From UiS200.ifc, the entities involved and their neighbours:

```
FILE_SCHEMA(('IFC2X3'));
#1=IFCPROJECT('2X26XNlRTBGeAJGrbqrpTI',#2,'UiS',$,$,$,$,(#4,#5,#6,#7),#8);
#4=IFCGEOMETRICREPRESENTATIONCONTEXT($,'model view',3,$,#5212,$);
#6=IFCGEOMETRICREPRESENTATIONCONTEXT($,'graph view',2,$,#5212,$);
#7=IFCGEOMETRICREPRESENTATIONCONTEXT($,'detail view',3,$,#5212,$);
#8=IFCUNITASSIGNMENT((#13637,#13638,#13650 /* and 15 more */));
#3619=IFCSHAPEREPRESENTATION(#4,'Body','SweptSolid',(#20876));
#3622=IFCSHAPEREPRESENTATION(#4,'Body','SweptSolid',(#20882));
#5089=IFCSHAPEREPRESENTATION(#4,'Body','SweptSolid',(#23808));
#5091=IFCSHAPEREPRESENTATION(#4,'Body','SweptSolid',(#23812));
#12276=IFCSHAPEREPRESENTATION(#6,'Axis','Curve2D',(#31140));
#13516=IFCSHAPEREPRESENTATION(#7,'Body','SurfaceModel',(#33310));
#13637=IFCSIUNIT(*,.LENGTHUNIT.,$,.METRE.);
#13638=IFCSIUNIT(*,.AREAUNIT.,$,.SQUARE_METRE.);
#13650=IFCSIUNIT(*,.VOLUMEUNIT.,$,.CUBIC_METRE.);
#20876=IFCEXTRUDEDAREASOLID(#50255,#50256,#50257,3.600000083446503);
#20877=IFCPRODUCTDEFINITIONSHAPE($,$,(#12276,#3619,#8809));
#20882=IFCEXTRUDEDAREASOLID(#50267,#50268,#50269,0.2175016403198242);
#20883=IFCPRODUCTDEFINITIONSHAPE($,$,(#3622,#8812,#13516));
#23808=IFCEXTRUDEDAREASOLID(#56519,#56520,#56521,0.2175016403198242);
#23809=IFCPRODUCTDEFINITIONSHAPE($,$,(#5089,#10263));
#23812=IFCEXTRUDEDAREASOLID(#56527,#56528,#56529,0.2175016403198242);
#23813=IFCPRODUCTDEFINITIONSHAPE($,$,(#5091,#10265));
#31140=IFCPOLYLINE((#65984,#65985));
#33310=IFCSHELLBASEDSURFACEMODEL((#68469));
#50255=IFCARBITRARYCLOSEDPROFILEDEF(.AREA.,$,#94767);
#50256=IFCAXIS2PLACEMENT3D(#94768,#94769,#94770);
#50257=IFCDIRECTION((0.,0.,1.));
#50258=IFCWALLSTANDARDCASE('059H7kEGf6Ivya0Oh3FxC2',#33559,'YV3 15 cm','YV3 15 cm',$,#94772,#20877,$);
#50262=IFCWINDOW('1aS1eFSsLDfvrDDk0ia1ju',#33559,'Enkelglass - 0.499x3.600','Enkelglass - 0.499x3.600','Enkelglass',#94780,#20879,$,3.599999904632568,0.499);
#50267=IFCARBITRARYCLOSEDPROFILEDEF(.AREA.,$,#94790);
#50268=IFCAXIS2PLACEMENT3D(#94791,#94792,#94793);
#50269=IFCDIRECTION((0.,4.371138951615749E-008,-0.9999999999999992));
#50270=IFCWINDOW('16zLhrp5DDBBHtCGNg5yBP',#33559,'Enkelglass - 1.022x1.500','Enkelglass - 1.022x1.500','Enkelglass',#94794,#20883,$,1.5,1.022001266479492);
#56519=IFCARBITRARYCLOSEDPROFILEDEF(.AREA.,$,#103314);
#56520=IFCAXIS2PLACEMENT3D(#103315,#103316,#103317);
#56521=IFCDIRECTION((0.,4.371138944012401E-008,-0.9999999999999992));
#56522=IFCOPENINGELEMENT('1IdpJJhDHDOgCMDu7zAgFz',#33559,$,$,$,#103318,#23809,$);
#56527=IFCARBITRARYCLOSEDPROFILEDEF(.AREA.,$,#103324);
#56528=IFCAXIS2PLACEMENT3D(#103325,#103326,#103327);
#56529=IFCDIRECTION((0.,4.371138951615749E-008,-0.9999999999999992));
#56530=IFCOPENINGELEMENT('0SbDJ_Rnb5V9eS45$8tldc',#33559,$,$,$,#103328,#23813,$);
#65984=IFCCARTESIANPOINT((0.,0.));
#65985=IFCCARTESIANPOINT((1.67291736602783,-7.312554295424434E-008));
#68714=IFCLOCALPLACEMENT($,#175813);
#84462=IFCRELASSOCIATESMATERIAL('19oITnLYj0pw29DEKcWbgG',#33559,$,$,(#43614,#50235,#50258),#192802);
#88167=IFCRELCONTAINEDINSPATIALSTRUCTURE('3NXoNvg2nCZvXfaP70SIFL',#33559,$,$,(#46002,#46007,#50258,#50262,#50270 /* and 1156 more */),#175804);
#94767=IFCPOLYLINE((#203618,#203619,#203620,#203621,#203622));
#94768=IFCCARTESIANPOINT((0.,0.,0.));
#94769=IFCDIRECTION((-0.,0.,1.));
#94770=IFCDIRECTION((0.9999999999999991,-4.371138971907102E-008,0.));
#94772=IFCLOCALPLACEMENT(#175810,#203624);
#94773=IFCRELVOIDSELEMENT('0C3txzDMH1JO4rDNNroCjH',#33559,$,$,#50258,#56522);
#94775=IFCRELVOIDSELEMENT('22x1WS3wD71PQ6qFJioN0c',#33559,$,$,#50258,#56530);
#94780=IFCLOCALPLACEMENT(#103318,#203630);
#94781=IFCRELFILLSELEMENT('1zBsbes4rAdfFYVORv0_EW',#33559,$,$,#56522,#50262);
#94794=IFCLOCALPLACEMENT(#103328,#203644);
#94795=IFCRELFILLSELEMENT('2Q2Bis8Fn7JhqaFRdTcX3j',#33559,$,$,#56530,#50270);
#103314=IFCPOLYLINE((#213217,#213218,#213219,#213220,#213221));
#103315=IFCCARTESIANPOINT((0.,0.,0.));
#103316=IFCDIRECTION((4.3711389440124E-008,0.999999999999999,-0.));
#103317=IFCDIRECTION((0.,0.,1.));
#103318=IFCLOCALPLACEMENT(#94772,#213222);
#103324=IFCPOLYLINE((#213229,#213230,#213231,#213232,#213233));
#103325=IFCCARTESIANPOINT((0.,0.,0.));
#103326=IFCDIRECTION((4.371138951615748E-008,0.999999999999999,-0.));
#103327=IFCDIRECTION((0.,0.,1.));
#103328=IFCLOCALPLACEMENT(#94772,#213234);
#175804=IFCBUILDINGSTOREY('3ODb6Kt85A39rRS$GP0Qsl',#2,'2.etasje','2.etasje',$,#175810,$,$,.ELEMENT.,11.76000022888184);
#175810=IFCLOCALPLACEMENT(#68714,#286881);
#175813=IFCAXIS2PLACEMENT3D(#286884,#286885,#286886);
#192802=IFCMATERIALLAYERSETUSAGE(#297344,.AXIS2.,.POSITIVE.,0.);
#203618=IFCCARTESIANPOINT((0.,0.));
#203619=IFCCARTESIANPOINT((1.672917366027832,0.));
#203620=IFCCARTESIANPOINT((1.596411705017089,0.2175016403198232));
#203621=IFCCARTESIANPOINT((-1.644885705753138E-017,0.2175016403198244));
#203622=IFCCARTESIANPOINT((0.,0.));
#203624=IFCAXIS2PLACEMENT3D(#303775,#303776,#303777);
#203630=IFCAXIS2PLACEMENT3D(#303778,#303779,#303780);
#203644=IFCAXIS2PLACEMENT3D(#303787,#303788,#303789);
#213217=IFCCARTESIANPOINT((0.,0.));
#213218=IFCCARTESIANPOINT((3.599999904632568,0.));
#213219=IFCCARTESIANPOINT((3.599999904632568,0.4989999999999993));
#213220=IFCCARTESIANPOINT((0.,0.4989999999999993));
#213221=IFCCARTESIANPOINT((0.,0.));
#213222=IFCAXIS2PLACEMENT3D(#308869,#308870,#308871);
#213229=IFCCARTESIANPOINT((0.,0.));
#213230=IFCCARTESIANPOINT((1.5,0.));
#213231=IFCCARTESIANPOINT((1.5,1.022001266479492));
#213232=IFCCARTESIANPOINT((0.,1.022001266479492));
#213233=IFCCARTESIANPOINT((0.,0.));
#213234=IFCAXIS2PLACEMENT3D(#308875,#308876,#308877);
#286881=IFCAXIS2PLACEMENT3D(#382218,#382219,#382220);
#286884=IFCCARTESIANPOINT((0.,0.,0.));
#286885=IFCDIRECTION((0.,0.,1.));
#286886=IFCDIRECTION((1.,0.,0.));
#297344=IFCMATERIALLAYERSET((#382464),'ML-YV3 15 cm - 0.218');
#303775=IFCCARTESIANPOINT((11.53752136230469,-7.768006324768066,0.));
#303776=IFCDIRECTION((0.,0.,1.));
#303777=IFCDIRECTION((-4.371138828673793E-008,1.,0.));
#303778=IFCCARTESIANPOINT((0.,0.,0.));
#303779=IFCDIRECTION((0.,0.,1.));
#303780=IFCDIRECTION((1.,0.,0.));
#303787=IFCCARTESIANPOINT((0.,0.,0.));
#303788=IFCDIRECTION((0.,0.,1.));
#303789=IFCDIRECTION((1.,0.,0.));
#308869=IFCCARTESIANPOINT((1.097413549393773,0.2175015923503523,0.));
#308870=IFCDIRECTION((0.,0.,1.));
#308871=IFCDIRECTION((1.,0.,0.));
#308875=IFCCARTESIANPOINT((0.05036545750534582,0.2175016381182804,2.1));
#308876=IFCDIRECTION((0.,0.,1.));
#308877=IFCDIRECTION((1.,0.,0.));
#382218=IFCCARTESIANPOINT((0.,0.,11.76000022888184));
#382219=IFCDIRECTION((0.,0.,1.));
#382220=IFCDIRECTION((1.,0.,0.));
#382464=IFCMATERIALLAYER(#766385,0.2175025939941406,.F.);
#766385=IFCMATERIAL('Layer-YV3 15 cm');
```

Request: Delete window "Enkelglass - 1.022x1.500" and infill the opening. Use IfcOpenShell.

```python
import ifcopenshell
import ifcopenshell.api.feature
import ifcopenshell.api.root
import ifcopenshell.geom
import ifcopenshell.util.shape

model = ifcopenshell.open("UiS200.ifc")
settings = ifcopenshell.geom.settings()


def volume(element):
    """Net volume in cubic metres, openings subtracted."""
    shape = ifcopenshell.geom.create_shape(settings, element)
    return ifcopenshell.util.shape.get_volume(shape.geometry)


window = model.by_id(50270)
opening = window.FillsVoids[0].RelatingOpeningElement
wall = opening.VoidsElements[0].RelatingBuildingElement
before = volume(wall)

ifcopenshell.api.root.remove_product(model, product=window)
ifcopenshell.api.feature.remove_feature(model, feature=opening)

after = volume(wall)

print(f"wall volume {before:.3f} -> {after:.3f} m3")

model.write("UiS200-out.ifc")
```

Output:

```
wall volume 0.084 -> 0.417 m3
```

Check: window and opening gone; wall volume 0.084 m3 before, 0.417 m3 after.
